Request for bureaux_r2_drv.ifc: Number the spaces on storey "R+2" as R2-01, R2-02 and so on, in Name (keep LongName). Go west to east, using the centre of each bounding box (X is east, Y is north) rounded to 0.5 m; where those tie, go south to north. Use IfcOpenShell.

First a look at what the model holds.

```python
import ifcopenshell
import ifcopenshell.util.element
import ifcopenshell.util.placement

model = ifcopenshell.open("bureaux_r2_drv.ifc")
print(model.schema)
storey = next(s for s in model.by_type("IfcBuildingStorey") if s.Name == "R+2")
spaces = [e for e in ifcopenshell.util.element.get_decomposition(storey) if e.is_a("IfcSpace")]
for e in sorted(spaces, key=lambda e: e.id()):
    origin = ifcopenshell.util.placement.get_local_placement(e.ObjectPlacement)[:3, 3]
    print(e.id(), e.Name, e.LongName, origin.round(2) + 0.0, sep=" | ")
```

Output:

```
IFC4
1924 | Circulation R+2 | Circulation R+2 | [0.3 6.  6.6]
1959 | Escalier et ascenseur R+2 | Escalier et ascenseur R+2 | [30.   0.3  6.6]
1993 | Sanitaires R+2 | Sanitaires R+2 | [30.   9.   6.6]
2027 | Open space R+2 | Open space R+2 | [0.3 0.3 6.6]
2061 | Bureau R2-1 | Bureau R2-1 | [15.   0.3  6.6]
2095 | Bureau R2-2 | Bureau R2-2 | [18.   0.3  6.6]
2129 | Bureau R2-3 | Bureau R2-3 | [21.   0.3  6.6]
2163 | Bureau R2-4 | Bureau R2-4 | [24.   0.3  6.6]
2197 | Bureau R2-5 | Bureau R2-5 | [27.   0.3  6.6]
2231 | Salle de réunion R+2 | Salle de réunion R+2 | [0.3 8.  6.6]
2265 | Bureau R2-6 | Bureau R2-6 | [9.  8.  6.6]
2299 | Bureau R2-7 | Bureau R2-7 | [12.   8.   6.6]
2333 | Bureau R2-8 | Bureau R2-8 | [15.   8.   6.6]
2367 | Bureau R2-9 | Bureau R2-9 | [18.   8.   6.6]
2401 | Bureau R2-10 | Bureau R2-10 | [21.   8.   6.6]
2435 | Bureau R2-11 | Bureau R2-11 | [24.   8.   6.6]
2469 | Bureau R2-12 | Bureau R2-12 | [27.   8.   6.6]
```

```python
import ifcopenshell
import ifcopenshell.geom
import ifcopenshell.util.element
import ifcopenshell.util.shape

model = ifcopenshell.open("bureaux_r2_drv.ifc")
settings = ifcopenshell.geom.settings()
settings.set("use-world-coords", True)


def centre(element):
    shape = ifcopenshell.geom.create_shape(settings, element)
    return ifcopenshell.util.shape.get_bbox_centroid(shape.geometry)


storey = next(s for s in model.by_type("IfcBuildingStorey") if s.Name == "R+2")
spaces = [e for e in ifcopenshell.util.element.get_decomposition(storey) if e.is_a("IfcSpace")]

# Insertion points can sit at a corner or the storey origin, so sort by the geometry (in metres).
centres = {e: centre(e) for e in spaces}
spaces.sort(key=lambda e: (round(centres[e][0] / 0.5), centres[e][1]))

for i, e in enumerate(spaces, start=1):
    number = f"R2-{i:02d}"
    e.Name = number
    print(e.id(), number)

model.write("bureaux_r2_drv_v2.ifc")
```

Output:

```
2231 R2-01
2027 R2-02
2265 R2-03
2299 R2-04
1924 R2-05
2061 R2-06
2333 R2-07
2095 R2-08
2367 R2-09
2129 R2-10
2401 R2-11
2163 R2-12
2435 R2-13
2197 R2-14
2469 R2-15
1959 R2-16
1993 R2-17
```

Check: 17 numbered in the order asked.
